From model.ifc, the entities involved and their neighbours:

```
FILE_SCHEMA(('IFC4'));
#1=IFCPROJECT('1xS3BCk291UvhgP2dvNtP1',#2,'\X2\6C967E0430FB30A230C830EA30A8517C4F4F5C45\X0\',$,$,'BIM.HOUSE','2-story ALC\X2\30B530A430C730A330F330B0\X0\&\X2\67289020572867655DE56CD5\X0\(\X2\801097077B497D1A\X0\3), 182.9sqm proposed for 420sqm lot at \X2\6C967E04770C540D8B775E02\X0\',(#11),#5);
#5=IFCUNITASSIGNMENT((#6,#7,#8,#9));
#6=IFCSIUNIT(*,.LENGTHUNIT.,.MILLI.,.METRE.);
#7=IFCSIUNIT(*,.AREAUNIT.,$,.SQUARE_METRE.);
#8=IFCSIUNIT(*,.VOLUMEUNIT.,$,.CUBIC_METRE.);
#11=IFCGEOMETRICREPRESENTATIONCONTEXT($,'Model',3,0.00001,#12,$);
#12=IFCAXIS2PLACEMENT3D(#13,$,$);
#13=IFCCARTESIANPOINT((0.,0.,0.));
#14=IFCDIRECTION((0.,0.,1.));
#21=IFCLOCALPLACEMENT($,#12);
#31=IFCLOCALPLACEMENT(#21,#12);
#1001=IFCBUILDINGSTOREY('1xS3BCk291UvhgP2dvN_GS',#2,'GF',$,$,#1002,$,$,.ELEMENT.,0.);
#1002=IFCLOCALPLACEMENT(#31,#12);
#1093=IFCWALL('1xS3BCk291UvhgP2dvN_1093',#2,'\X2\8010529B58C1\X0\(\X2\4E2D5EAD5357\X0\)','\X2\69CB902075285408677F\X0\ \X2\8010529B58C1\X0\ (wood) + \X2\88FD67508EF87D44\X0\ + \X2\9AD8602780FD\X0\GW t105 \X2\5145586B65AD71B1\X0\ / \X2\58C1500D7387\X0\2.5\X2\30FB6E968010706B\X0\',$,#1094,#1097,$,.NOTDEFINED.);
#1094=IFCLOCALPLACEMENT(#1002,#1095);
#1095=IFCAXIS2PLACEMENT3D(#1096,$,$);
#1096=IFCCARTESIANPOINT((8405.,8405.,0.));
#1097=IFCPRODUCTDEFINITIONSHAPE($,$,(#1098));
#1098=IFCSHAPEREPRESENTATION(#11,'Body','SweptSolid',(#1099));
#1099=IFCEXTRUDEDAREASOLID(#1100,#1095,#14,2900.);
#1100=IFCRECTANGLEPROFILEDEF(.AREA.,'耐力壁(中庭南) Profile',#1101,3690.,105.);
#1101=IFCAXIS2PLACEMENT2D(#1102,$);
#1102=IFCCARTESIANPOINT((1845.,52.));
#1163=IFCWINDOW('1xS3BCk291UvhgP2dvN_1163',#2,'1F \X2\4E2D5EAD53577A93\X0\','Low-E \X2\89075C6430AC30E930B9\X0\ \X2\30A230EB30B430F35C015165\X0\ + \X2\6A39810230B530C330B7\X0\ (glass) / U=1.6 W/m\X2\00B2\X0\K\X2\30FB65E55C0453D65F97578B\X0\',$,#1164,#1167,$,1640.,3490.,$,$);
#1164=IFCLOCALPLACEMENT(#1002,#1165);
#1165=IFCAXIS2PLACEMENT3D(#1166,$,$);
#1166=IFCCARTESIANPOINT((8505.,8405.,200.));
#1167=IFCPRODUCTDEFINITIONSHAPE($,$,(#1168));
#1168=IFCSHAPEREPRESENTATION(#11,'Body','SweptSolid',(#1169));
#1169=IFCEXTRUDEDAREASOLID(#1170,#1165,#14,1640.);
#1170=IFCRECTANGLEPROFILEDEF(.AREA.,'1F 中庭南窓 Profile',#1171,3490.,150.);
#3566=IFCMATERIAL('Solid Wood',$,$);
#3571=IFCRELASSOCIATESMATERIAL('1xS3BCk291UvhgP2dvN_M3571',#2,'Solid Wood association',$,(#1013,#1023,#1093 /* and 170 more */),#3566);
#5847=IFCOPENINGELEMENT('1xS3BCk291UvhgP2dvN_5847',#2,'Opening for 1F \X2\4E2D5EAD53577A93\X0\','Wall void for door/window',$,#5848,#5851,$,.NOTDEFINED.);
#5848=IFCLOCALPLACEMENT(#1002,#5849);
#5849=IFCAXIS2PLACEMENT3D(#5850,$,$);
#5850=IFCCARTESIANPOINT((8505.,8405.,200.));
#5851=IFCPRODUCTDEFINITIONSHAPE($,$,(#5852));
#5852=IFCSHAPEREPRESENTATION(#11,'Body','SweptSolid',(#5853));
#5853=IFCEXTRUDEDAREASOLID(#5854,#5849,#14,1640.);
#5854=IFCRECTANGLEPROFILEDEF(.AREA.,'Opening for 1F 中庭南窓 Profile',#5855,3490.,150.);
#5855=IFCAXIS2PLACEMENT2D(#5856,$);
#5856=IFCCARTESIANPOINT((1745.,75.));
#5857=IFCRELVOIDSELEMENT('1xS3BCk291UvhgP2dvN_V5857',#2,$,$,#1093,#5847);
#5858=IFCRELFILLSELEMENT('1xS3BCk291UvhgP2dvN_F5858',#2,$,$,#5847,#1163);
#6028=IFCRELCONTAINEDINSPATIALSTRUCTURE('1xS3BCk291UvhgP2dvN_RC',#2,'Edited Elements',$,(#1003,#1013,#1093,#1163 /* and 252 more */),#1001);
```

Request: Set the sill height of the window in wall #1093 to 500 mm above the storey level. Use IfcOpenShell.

```python
import numpy as np
import ifcopenshell
import ifcopenshell.api.geometry
import ifcopenshell.geom
import ifcopenshell.util.element
import ifcopenshell.util.placement
import ifcopenshell.util.shape
import ifcopenshell.util.unit

model = ifcopenshell.open("model.ifc")
unit_scale = ifcopenshell.util.unit.calculate_unit_scale(model)

window = model.by_guid("1xS3BCk291UvhgP2dvN_1163")
opening = window.FillsVoids[0].RelatingOpeningElement
storey = ifcopenshell.util.element.get_container(window, ifc_class="IfcBuildingStorey")
level = ifcopenshell.util.placement.get_local_placement(storey.ObjectPlacement)[2, 3]

# The opening's origin need not be at the sill, so measure its lowest point.
shape = ifcopenshell.geom.create_shape(ifcopenshell.geom.settings(), opening)
bottom = ifcopenshell.util.shape.get_shape_bottom_elevation(shape, shape.geometry) / unit_scale
dz = level + 0.5 / unit_scale - bottom

shift = np.array([0.0, 0.0, dz])
# The window is not placed relative to its opening, so move both.
for product in (opening, window):
    matrix = ifcopenshell.util.placement.get_local_placement(product.ObjectPlacement)
    matrix[:3, 3] += shift
    ifcopenshell.api.geometry.edit_object_placement(model, product=product, matrix=matrix, is_si=False)

print(f"moved by {dz * unit_scale:+.3f} m")

model.write("model_rev.ifc")
```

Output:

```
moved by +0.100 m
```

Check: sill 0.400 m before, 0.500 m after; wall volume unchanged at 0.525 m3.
